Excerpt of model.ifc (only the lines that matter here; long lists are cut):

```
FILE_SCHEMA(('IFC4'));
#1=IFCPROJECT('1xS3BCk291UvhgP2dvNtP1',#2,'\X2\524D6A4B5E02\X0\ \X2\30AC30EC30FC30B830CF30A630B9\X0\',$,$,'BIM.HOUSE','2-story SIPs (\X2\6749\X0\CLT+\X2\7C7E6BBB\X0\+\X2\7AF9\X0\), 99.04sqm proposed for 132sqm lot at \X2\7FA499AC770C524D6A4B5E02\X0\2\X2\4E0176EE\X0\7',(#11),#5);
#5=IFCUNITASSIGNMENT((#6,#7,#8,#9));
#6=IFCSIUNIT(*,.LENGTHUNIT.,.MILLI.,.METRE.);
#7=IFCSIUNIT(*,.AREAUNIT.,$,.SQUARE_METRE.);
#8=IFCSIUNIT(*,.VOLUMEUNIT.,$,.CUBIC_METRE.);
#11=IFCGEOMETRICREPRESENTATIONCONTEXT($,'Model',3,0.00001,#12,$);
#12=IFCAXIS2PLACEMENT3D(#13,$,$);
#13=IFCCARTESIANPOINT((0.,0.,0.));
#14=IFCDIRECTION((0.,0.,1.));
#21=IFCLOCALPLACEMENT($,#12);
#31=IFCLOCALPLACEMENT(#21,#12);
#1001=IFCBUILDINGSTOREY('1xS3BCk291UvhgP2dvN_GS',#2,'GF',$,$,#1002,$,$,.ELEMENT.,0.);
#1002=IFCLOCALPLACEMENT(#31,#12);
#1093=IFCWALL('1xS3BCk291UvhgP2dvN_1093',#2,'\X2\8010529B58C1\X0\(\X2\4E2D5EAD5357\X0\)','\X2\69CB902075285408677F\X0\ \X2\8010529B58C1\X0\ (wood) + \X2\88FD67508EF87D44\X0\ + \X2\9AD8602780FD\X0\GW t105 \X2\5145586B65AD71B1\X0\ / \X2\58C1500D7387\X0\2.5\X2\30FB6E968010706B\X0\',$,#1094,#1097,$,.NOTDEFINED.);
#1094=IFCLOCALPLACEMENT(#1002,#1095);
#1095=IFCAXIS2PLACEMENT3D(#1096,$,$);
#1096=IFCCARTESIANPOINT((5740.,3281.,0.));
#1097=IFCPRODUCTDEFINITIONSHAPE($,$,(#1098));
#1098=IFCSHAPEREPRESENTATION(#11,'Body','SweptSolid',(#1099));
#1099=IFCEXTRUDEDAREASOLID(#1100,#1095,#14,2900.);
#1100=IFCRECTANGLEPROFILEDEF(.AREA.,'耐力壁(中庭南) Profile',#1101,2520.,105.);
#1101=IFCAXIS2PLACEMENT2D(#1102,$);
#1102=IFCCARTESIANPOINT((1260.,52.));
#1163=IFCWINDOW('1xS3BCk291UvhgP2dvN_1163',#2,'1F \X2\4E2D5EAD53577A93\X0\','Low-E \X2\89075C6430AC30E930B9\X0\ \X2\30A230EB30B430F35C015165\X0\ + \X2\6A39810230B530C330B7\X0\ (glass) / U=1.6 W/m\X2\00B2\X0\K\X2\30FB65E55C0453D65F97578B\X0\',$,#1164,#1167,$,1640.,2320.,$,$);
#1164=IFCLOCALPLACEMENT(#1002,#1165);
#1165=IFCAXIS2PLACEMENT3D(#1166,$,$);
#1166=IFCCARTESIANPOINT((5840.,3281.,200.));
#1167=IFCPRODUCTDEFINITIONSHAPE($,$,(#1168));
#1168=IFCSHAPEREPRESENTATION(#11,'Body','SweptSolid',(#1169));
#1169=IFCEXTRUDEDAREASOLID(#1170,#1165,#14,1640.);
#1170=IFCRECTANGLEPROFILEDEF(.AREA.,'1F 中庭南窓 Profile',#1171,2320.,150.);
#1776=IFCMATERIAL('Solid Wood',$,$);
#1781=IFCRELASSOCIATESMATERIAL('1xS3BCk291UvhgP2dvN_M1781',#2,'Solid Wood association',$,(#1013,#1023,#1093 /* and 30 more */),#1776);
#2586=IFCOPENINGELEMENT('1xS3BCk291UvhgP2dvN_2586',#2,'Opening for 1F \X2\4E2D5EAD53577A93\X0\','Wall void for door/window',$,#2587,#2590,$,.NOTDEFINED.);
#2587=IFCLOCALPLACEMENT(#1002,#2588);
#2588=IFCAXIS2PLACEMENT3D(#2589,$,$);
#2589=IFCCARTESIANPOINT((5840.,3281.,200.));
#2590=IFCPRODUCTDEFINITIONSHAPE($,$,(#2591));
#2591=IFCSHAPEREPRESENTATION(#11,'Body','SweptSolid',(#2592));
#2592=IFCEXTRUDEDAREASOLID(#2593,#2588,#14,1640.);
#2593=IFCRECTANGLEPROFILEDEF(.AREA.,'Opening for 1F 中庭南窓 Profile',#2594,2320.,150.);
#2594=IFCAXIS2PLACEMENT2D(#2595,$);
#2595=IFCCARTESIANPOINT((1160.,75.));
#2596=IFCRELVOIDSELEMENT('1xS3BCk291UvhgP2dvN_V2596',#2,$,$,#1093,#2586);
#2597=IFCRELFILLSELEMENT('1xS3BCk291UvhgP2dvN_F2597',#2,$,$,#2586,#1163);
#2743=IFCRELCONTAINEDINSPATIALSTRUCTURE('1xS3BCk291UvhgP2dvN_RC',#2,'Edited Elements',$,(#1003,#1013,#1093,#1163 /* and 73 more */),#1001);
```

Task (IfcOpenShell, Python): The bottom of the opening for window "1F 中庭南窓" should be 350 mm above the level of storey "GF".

```python
import numpy as np
import ifcopenshell
import ifcopenshell.api.geometry
import ifcopenshell.geom
import ifcopenshell.util.element
import ifcopenshell.util.placement
import ifcopenshell.util.shape
import ifcopenshell.util.unit

model = ifcopenshell.open("model.ifc")
unit_scale = ifcopenshell.util.unit.calculate_unit_scale(model)

window = model.by_guid("1xS3BCk291UvhgP2dvN_1163")
opening = window.FillsVoids[0].RelatingOpeningElement
storey = ifcopenshell.util.element.get_container(window, ifc_class="IfcBuildingStorey")
level = ifcopenshell.util.placement.get_local_placement(storey.ObjectPlacement)[2, 3]

# The opening's origin need not be at the sill, so measure its lowest point.
shape = ifcopenshell.geom.create_shape(ifcopenshell.geom.settings(), opening)
bottom = ifcopenshell.util.shape.get_shape_bottom_elevation(shape, shape.geometry) / unit_scale
dz = level + 0.35 / unit_scale - bottom

shift = np.array([0.0, 0.0, dz])
# The window is not placed relative to its opening, so move both.
for product in (opening, window):
    matrix = ifcopenshell.util.placement.get_local_placement(product.ObjectPlacement)
    matrix[:3, 3] += shift
    ifcopenshell.api.geometry.edit_object_placement(model, product=product, matrix=matrix, is_si=False)

print(f"moved by {dz * unit_scale:+.3f} m")

model.write("model_updated.ifc")
```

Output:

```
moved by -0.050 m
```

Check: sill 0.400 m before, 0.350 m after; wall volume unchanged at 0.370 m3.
